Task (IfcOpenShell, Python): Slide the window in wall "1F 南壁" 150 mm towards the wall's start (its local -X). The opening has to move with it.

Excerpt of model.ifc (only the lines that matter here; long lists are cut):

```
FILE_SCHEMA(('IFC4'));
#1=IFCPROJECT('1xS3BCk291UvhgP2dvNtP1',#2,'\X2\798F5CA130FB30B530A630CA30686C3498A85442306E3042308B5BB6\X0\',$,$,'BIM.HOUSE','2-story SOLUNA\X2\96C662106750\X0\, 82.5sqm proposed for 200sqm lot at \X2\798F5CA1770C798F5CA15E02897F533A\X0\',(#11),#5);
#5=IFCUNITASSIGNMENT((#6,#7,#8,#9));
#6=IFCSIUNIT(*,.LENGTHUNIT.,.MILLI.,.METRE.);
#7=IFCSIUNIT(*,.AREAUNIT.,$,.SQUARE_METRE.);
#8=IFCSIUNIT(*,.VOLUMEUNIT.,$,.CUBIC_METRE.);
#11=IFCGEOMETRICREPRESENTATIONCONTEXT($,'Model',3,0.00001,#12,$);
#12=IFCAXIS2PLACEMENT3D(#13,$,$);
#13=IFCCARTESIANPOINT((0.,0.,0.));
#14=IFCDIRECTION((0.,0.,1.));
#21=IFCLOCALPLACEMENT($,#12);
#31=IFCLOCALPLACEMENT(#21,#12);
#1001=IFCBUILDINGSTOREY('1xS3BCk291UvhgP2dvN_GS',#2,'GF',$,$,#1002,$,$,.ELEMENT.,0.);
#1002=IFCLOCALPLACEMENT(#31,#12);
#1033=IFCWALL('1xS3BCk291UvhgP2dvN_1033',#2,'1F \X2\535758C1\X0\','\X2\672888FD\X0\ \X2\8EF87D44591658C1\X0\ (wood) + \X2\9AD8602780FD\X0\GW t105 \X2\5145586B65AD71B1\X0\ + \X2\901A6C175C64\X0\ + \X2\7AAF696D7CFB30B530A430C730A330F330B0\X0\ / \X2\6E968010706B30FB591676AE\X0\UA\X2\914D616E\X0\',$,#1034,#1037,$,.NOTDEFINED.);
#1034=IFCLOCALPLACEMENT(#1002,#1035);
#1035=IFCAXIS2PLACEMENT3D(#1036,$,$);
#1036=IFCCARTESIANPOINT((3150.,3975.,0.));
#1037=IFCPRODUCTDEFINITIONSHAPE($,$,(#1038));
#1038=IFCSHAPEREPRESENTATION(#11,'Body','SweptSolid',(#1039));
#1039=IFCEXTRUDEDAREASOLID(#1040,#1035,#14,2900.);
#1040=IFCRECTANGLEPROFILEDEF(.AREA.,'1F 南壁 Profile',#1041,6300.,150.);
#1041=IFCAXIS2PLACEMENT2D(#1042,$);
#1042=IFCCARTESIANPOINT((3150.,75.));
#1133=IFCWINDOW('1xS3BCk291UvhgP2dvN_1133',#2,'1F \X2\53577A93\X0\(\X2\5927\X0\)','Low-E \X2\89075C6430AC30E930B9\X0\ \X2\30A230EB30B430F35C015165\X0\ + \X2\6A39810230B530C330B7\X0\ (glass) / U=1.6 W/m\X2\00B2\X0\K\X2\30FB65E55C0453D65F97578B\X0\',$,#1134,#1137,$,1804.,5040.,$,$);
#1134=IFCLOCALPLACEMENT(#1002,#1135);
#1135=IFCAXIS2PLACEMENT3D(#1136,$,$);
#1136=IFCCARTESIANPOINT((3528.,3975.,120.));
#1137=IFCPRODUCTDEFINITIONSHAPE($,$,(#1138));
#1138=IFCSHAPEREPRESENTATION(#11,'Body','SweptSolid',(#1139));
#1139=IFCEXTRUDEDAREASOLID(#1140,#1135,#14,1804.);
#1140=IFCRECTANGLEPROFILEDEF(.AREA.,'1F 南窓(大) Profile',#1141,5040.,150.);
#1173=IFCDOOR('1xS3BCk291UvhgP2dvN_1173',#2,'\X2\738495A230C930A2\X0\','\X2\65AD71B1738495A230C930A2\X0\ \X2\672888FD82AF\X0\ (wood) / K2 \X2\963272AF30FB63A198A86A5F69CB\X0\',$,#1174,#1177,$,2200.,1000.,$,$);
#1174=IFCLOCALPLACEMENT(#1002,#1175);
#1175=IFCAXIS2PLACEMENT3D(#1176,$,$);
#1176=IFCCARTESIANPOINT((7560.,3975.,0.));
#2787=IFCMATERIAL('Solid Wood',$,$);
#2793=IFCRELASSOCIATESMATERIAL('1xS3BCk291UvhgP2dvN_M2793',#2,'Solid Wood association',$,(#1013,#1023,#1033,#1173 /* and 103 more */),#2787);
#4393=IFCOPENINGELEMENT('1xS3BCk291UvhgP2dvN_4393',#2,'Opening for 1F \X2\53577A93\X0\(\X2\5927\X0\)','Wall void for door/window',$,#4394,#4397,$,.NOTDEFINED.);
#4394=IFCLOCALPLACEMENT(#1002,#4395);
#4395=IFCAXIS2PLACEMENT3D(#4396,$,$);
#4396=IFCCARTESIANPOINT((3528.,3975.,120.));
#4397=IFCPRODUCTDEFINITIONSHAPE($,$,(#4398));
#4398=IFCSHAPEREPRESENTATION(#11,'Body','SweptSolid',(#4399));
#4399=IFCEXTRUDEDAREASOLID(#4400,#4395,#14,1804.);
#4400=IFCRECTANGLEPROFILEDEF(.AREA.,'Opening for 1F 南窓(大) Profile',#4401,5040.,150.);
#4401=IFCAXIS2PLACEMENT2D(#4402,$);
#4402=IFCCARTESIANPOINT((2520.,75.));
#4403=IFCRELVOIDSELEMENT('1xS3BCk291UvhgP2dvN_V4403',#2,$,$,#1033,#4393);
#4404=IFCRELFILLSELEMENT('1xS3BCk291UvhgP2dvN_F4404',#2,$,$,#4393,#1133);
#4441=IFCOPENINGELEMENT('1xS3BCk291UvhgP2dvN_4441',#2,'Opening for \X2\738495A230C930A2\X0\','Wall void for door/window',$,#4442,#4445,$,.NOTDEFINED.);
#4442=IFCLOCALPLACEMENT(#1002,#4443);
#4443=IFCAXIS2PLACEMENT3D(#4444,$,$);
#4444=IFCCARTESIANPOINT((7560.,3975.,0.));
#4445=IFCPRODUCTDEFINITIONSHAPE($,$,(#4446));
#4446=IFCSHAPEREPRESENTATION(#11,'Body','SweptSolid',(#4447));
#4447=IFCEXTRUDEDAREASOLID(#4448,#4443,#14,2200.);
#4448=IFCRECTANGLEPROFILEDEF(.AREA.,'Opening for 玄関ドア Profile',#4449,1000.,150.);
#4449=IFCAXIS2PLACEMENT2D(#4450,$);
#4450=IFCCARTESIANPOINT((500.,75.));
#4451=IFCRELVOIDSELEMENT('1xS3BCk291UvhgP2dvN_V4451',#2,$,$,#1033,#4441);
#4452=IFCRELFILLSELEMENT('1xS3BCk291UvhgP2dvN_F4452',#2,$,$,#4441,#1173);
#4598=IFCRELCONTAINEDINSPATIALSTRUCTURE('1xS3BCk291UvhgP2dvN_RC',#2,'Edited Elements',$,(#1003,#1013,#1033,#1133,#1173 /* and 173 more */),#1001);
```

```python
import ifcopenshell
import ifcopenshell.api.geometry
import ifcopenshell.util.placement

model = ifcopenshell.open("model.ifc")

window = model.by_id(1133)
opening = window.FillsVoids[0].RelatingOpeningElement
wall = opening.VoidsElements[0].RelatingBuildingElement

wall_matrix = ifcopenshell.util.placement.get_local_placement(wall.ObjectPlacement)
shift = wall_matrix[:3, 0] * -150.0
before = ifcopenshell.util.placement.get_local_placement(window.ObjectPlacement)[:3, 3].copy()

# The window is not placed relative to its opening, so move both.
for product in (opening, window):
    matrix = ifcopenshell.util.placement.get_local_placement(product.ObjectPlacement)
    matrix[:3, 3] += shift
    ifcopenshell.api.geometry.edit_object_placement(model, product=product, matrix=matrix, is_si=False)

after = ifcopenshell.util.placement.get_local_placement(window.ObjectPlacement)[:3, 3]
print("window moved by", (after - before).round(3) + 0.0)

model.write("model-out.ifc")
```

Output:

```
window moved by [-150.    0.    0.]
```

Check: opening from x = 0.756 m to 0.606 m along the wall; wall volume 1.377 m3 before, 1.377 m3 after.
